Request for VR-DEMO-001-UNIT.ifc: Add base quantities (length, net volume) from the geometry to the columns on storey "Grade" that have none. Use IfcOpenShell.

First a look at what the model holds.

```python
import ifcopenshell
import ifcopenshell.util.element
import ifcopenshell.util.unit

model = ifcopenshell.open("VR-DEMO-001-UNIT.ifc")
print(model.schema)
for unit_type in ("LENGTHUNIT", "AREAUNIT", "VOLUMEUNIT"):
    print(unit_type, ifcopenshell.util.unit.calculate_unit_scale(model, unit_type))
storey = next(s for s in model.by_type("IfcBuildingStorey") if s.Name == "Grade")
columns = [e for e in ifcopenshell.util.element.get_decomposition(storey) if e.is_a("IfcColumn")]
for e in sorted(columns, key=lambda e: e.id()):
    print(e.id(), e.is_a(), e.Name, list(ifcopenshell.util.element.get_psets(e, qtos_only=True)), sep=" | ")
```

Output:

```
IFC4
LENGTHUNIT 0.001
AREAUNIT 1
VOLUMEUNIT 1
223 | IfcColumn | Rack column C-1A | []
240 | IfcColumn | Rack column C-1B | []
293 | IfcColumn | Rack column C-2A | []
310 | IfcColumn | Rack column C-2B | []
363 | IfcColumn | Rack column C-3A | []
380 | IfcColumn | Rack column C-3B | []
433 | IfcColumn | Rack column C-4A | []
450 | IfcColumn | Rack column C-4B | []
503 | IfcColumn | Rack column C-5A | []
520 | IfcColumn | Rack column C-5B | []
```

```python
import ifcopenshell
import ifcopenshell.api.pset
import ifcopenshell.geom
import ifcopenshell.util.element
import ifcopenshell.util.shape
import ifcopenshell.util.unit

model = ifcopenshell.open("VR-DEMO-001-UNIT.ifc")
unit_scale = ifcopenshell.util.unit.calculate_unit_scale(model)
volume_scale = ifcopenshell.util.unit.calculate_unit_scale(model, "VOLUMEUNIT")
settings = ifcopenshell.geom.settings()

storey = next(s for s in model.by_type("IfcBuildingStorey") if s.Name == "Grade")
columns = [e for e in ifcopenshell.util.element.get_decomposition(storey) if e.is_a("IfcColumn")]

for e in sorted(columns, key=lambda e: e.id()):
    if ifcopenshell.util.element.get_psets(e, qtos_only=True, should_inherit=False):
        continue
    # Geometry comes back in metres, in the element's own axes.
    shape = ifcopenshell.geom.create_shape(settings, e)
    values = {
        "Length": ifcopenshell.util.shape.get_z(shape.geometry) / unit_scale,
        "NetVolume": ifcopenshell.util.shape.get_volume(shape.geometry) / volume_scale,
    }
    qto = ifcopenshell.api.pset.add_qto(model, product=e, name="Qto_ColumnBaseQuantities")
    ifcopenshell.api.pset.edit_qto(model, qto=qto, properties=values)
    print(e.id(), {k: round(v, 3) for k, v in values.items()})

model.write("VR-DEMO-001-UNIT_updated.ifc")
```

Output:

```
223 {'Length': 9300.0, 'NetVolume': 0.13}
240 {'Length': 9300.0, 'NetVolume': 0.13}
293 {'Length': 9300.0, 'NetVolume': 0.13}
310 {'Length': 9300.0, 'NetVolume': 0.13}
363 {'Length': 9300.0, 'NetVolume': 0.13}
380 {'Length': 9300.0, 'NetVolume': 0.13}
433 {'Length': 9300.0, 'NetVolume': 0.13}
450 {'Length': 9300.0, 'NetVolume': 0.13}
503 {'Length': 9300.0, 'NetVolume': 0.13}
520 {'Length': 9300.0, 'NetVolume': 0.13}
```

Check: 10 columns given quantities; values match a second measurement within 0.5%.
